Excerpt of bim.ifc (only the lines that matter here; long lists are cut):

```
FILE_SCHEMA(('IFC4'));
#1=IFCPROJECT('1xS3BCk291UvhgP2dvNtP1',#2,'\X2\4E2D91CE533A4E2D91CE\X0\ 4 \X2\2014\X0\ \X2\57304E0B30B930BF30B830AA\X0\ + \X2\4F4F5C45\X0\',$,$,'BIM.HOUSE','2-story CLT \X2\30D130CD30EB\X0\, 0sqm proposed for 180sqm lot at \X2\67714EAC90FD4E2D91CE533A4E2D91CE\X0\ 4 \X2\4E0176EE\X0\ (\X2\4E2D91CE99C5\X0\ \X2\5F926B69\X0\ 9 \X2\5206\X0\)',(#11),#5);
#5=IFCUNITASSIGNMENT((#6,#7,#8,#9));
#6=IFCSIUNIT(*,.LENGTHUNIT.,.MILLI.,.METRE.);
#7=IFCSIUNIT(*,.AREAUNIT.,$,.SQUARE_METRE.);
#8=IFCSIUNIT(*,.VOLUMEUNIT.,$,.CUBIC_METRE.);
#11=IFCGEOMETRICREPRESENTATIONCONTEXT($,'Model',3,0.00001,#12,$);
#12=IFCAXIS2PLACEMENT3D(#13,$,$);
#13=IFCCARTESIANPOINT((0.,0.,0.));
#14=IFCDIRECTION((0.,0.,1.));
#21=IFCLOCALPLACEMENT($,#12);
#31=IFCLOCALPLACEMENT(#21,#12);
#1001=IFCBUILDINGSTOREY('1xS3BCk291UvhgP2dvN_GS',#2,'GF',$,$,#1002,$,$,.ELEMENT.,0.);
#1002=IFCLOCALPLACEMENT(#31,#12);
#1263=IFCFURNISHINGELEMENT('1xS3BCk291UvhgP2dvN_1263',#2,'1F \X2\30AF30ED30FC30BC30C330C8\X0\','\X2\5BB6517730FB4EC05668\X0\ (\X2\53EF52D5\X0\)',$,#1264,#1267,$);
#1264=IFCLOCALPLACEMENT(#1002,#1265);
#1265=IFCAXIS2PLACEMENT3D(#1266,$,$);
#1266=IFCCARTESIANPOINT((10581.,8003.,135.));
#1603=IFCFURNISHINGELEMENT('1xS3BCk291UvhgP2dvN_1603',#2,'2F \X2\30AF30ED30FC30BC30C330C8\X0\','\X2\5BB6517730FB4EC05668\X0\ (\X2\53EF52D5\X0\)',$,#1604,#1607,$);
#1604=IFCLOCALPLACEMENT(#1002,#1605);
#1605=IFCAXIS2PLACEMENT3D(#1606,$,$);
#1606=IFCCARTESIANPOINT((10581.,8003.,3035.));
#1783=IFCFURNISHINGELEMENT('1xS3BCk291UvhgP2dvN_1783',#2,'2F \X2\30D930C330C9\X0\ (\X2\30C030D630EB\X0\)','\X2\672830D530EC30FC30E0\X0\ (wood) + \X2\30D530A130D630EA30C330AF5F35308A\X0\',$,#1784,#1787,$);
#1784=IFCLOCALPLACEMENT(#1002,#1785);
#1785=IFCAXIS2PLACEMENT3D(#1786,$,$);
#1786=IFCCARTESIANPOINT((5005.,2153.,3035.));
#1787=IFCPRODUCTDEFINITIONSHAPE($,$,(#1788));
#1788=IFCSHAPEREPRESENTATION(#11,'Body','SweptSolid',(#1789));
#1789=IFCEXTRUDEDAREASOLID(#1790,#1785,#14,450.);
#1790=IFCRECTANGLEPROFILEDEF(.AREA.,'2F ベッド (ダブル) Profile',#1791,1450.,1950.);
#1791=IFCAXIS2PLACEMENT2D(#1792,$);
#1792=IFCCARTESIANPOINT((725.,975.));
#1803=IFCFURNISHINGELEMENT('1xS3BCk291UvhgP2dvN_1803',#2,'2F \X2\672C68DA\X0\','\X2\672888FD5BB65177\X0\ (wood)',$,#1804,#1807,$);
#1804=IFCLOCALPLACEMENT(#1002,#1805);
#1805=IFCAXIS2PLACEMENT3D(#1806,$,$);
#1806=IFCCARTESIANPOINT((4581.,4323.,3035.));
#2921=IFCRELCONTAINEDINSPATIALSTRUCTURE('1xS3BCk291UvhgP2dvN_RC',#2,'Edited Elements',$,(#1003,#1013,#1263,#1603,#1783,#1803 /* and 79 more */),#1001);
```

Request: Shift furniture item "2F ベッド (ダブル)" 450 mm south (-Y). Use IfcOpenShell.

```python
import ifcopenshell
import ifcopenshell.api.geometry
import ifcopenshell.util.placement
import ifcopenshell.util.unit

model = ifcopenshell.open("bim.ifc")
unit_scale = ifcopenshell.util.unit.calculate_unit_scale(model)

item = model.by_guid("1xS3BCk291UvhgP2dvN_1783")
matrix = ifcopenshell.util.placement.get_local_placement(item.ObjectPlacement)
matrix[1, 3] -= 0.45 / unit_scale
ifcopenshell.api.geometry.edit_object_placement(model, product=item, matrix=matrix, is_si=False)

print(ifcopenshell.util.placement.get_local_placement(item.ObjectPlacement).round(3) + 0.0)

model.write("bim_v2.ifc")
```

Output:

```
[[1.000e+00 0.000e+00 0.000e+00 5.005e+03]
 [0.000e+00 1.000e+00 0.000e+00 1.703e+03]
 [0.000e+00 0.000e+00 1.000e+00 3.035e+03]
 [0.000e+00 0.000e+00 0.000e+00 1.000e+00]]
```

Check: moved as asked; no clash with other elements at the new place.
